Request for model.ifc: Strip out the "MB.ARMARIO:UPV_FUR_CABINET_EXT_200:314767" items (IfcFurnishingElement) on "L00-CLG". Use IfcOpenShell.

First a look at what the model holds.

```python
import ifcopenshell
import ifcopenshell.util.element

model = ifcopenshell.open("model.ifc")
print(model.schema)
storey = next(s for s in model.by_type("IfcBuildingStorey") if s.Name == "L00-CLG")
furniture = [e for e in ifcopenshell.util.element.get_decomposition(storey) if e.is_a("IfcFurnishingElement")]
seen = {}
for e in furniture:
    element_type = ifcopenshell.util.element.get_type(e)
    name = element_type.Name if element_type not in (None, e) else None
    seen[name] = seen.get(name, 0) + 1
for name, count in sorted(seen.items(), key=str):
    print(count, "x", name)
```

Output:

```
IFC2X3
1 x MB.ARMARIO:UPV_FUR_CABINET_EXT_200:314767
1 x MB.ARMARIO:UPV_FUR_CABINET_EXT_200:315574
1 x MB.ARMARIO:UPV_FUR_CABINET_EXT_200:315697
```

```python
import ifcopenshell
import ifcopenshell.api.root
import ifcopenshell.util.element

model = ifcopenshell.open("model.ifc")

storey = next(s for s in model.by_type("IfcBuildingStorey") if s.Name == "L00-CLG")
furniture = [e for e in ifcopenshell.util.element.get_decomposition(storey) if e.is_a("IfcFurnishingElement")]
targets = [e for e in furniture if (t := ifcopenshell.util.element.get_type(e)) not in (None, e) and t.Name == "MB.ARMARIO:UPV_FUR_CABINET_EXT_200:314767"]

for e in targets:
    ifcopenshell.api.root.remove_product(model, product=e)
print(len(targets), "removed")

model.write("model_v2.ifc")
```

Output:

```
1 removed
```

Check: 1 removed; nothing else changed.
